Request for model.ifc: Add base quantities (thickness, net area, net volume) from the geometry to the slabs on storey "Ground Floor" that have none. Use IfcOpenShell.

First a look at what the model holds.

```python
import ifcopenshell
import ifcopenshell.util.element
import ifcopenshell.util.unit

model = ifcopenshell.open("model.ifc")
print(model.schema)
for unit_type in ("LENGTHUNIT", "AREAUNIT", "VOLUMEUNIT"):
    print(unit_type, ifcopenshell.util.unit.calculate_unit_scale(model, unit_type))
storey = next(s for s in model.by_type("IfcBuildingStorey") if s.Name == "Ground Floor")
slabs = [e for e in ifcopenshell.util.element.get_decomposition(storey) if e.is_a("IfcSlab")]
for e in sorted(slabs, key=lambda e: e.id()):
    print(e.id(), e.is_a(), e.Name, list(ifcopenshell.util.element.get_psets(e, qtos_only=True)), sep=" | ")
```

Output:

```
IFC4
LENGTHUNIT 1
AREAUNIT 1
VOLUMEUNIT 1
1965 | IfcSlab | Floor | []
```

```python
import ifcopenshell
import ifcopenshell.api.pset
import ifcopenshell.geom
import ifcopenshell.util.element
import ifcopenshell.util.shape
import ifcopenshell.util.unit

model = ifcopenshell.open("model.ifc")
unit_scale = ifcopenshell.util.unit.calculate_unit_scale(model)
area_scale = ifcopenshell.util.unit.calculate_unit_scale(model, "AREAUNIT")
volume_scale = ifcopenshell.util.unit.calculate_unit_scale(model, "VOLUMEUNIT")
settings = ifcopenshell.geom.settings()

storey = next(s for s in model.by_type("IfcBuildingStorey") if s.Name == "Ground Floor")
slabs = [e for e in ifcopenshell.util.element.get_decomposition(storey) if e.is_a("IfcSlab")]

for e in sorted(slabs, key=lambda e: e.id()):
    if ifcopenshell.util.element.get_psets(e, qtos_only=True, should_inherit=False):
        continue
    # Geometry comes back in metres, in the element's own axes.
    shape = ifcopenshell.geom.create_shape(settings, e)
    values = {
        "Width": ifcopenshell.util.shape.get_z(shape.geometry) / unit_scale,
        "NetArea": ifcopenshell.util.shape.get_footprint_area(shape.geometry) / area_scale,
        "NetVolume": ifcopenshell.util.shape.get_volume(shape.geometry) / volume_scale,
    }
    qto = ifcopenshell.api.pset.add_qto(model, product=e, name="Qto_SlabBaseQuantities")
    ifcopenshell.api.pset.edit_qto(model, qto=qto, properties=values)
    print(e.id(), {k: round(v, 3) for k, v in values.items()})

model.write("model_rev.ifc")
```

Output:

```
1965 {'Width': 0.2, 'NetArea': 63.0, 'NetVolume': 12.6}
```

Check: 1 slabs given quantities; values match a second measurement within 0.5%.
